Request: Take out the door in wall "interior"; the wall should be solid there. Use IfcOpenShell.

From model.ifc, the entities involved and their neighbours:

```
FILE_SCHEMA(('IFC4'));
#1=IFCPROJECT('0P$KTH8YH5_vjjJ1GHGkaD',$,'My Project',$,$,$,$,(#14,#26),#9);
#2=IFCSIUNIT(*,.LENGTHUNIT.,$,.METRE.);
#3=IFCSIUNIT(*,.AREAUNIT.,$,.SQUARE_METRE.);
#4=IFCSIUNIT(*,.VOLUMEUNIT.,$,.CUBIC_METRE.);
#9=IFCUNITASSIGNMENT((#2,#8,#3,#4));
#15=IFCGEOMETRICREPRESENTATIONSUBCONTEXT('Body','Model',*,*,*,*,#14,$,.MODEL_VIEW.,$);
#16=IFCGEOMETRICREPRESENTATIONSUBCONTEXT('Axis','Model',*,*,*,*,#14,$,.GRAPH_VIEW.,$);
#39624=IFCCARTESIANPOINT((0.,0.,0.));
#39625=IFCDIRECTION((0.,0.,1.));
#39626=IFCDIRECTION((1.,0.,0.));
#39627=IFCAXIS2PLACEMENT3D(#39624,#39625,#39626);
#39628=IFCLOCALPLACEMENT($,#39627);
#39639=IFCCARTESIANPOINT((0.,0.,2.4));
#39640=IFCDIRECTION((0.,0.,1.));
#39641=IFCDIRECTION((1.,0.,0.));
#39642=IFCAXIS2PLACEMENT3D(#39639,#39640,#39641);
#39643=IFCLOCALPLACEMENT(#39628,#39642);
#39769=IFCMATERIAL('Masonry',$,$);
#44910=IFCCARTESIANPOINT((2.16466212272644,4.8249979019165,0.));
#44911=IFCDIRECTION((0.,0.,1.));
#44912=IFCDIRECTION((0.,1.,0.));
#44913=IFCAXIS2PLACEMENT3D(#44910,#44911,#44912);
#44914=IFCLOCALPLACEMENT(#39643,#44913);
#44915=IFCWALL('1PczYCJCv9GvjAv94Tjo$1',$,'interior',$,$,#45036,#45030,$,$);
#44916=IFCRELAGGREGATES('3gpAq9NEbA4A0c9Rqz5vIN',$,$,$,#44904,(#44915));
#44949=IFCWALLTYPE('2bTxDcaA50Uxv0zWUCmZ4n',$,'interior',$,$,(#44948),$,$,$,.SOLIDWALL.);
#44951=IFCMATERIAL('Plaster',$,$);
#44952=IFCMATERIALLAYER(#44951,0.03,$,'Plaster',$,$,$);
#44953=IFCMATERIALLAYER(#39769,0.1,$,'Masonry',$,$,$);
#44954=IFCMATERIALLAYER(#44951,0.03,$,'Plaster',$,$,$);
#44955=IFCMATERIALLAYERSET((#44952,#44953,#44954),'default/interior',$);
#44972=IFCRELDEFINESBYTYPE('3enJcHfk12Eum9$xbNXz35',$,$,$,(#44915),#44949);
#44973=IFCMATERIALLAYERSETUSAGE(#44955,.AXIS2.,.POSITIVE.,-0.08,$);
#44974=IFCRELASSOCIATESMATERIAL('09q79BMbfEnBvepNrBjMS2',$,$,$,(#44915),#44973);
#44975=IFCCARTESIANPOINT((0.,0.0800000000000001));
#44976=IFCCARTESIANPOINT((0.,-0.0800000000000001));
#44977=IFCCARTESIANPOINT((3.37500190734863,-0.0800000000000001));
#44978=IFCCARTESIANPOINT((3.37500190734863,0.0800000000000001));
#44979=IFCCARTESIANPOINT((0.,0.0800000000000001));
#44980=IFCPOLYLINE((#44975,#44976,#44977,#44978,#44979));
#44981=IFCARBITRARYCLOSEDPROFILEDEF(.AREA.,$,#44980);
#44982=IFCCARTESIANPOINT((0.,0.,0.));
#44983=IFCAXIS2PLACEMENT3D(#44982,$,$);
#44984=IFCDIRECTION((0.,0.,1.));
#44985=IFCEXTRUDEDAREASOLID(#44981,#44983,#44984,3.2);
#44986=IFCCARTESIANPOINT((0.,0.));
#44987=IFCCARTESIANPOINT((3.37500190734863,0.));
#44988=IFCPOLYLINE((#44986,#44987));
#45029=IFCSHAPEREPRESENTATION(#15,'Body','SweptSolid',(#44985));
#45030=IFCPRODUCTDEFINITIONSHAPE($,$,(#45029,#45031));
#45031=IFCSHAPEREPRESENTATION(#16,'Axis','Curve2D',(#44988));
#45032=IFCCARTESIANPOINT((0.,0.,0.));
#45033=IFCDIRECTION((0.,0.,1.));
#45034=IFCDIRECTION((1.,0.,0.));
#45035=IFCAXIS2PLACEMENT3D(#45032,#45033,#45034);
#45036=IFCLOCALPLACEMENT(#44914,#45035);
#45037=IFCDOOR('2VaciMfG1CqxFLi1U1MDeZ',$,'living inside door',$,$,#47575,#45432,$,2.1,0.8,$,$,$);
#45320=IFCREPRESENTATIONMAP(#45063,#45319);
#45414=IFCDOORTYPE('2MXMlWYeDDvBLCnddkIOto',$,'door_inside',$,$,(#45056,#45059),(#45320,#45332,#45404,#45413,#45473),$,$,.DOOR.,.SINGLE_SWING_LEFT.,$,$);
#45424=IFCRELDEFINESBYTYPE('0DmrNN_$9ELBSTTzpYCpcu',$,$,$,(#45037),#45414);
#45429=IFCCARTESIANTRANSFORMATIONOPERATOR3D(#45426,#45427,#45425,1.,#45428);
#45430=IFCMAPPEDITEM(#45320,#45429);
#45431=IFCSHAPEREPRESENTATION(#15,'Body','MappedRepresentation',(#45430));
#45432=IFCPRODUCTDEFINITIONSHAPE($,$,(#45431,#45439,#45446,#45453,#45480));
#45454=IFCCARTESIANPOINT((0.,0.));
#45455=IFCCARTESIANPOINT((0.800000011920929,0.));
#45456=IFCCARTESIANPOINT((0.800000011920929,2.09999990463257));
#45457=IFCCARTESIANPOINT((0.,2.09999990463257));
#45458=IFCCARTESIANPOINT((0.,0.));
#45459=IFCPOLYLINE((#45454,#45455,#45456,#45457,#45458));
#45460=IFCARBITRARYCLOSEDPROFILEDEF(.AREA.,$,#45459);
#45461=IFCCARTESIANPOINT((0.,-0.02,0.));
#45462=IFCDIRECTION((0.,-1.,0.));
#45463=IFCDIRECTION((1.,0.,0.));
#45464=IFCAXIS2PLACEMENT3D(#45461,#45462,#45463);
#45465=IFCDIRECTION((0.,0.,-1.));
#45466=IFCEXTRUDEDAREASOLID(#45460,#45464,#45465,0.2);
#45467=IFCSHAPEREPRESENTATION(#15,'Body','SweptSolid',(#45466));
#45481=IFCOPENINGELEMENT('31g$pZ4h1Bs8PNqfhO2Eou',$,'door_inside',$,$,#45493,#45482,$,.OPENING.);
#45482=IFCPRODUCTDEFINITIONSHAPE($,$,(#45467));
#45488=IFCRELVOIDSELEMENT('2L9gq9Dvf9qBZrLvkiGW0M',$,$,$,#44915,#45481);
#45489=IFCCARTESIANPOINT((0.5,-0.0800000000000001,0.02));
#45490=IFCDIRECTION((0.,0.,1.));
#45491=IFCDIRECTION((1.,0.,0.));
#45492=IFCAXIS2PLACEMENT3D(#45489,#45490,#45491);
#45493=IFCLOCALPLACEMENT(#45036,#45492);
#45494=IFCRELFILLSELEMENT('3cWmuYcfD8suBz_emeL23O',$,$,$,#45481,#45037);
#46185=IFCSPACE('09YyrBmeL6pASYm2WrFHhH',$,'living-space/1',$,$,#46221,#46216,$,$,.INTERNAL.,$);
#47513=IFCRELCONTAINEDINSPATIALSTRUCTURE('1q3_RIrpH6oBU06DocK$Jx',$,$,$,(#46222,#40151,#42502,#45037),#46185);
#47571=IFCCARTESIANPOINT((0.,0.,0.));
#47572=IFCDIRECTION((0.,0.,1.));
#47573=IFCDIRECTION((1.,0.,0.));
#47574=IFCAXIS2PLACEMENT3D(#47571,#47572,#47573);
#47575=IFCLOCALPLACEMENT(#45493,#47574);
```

```python
import ifcopenshell
import ifcopenshell.api.feature
import ifcopenshell.api.root
import ifcopenshell.geom
import ifcopenshell.util.shape

model = ifcopenshell.open("model.ifc")
settings = ifcopenshell.geom.settings()


def volume(element):
    """Net volume in cubic metres, openings subtracted."""
    shape = ifcopenshell.geom.create_shape(settings, element)
    return ifcopenshell.util.shape.get_volume(shape.geometry)


door = model.by_guid("2VaciMfG1CqxFLi1U1MDeZ")
opening = door.FillsVoids[0].RelatingOpeningElement
wall = opening.VoidsElements[0].RelatingBuildingElement
before = volume(wall)

ifcopenshell.api.root.remove_product(model, product=door)
ifcopenshell.api.feature.remove_feature(model, feature=opening)

after = volume(wall)

print(f"wall volume {before:.3f} -> {after:.3f} m3")

model.write("model_rev.ifc")
```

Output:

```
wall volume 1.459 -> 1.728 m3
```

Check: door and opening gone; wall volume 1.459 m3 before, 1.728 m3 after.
